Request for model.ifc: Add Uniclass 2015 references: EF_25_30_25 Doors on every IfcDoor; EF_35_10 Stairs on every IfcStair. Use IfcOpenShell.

First a look at what the model holds.

```python
import ifcopenshell

model = ifcopenshell.open("model.ifc")
print(model.schema)
print("classifications:", [c.Name for c in model.by_type("IfcClassification")])
for ifc_class in ("IfcDoor", "IfcRoof", "IfcStair", "IfcWall", "IfcWindow"):
    print(ifc_class, len(model.by_type(ifc_class)))
```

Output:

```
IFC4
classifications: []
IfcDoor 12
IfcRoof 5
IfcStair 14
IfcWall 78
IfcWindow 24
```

```python
import ifcopenshell
import ifcopenshell.api.classification

model = ifcopenshell.open("model.ifc")

system = ifcopenshell.api.classification.add_classification(model, classification="Uniclass 2015")

codes = {
    "IfcDoor": ("EF_25_30_25", "Doors"),
    "IfcStair": ("EF_35_10", "Stairs"),
}
for ifc_class, (code, name) in codes.items():
    products = model.by_type(ifc_class)
    ifcopenshell.api.classification.add_reference(
        model, products=products, classification=system, identification=code, name=name
    )
    print(code, len(products))

model.write("model_v2.ifc")
```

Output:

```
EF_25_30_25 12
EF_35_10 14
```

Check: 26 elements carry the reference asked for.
